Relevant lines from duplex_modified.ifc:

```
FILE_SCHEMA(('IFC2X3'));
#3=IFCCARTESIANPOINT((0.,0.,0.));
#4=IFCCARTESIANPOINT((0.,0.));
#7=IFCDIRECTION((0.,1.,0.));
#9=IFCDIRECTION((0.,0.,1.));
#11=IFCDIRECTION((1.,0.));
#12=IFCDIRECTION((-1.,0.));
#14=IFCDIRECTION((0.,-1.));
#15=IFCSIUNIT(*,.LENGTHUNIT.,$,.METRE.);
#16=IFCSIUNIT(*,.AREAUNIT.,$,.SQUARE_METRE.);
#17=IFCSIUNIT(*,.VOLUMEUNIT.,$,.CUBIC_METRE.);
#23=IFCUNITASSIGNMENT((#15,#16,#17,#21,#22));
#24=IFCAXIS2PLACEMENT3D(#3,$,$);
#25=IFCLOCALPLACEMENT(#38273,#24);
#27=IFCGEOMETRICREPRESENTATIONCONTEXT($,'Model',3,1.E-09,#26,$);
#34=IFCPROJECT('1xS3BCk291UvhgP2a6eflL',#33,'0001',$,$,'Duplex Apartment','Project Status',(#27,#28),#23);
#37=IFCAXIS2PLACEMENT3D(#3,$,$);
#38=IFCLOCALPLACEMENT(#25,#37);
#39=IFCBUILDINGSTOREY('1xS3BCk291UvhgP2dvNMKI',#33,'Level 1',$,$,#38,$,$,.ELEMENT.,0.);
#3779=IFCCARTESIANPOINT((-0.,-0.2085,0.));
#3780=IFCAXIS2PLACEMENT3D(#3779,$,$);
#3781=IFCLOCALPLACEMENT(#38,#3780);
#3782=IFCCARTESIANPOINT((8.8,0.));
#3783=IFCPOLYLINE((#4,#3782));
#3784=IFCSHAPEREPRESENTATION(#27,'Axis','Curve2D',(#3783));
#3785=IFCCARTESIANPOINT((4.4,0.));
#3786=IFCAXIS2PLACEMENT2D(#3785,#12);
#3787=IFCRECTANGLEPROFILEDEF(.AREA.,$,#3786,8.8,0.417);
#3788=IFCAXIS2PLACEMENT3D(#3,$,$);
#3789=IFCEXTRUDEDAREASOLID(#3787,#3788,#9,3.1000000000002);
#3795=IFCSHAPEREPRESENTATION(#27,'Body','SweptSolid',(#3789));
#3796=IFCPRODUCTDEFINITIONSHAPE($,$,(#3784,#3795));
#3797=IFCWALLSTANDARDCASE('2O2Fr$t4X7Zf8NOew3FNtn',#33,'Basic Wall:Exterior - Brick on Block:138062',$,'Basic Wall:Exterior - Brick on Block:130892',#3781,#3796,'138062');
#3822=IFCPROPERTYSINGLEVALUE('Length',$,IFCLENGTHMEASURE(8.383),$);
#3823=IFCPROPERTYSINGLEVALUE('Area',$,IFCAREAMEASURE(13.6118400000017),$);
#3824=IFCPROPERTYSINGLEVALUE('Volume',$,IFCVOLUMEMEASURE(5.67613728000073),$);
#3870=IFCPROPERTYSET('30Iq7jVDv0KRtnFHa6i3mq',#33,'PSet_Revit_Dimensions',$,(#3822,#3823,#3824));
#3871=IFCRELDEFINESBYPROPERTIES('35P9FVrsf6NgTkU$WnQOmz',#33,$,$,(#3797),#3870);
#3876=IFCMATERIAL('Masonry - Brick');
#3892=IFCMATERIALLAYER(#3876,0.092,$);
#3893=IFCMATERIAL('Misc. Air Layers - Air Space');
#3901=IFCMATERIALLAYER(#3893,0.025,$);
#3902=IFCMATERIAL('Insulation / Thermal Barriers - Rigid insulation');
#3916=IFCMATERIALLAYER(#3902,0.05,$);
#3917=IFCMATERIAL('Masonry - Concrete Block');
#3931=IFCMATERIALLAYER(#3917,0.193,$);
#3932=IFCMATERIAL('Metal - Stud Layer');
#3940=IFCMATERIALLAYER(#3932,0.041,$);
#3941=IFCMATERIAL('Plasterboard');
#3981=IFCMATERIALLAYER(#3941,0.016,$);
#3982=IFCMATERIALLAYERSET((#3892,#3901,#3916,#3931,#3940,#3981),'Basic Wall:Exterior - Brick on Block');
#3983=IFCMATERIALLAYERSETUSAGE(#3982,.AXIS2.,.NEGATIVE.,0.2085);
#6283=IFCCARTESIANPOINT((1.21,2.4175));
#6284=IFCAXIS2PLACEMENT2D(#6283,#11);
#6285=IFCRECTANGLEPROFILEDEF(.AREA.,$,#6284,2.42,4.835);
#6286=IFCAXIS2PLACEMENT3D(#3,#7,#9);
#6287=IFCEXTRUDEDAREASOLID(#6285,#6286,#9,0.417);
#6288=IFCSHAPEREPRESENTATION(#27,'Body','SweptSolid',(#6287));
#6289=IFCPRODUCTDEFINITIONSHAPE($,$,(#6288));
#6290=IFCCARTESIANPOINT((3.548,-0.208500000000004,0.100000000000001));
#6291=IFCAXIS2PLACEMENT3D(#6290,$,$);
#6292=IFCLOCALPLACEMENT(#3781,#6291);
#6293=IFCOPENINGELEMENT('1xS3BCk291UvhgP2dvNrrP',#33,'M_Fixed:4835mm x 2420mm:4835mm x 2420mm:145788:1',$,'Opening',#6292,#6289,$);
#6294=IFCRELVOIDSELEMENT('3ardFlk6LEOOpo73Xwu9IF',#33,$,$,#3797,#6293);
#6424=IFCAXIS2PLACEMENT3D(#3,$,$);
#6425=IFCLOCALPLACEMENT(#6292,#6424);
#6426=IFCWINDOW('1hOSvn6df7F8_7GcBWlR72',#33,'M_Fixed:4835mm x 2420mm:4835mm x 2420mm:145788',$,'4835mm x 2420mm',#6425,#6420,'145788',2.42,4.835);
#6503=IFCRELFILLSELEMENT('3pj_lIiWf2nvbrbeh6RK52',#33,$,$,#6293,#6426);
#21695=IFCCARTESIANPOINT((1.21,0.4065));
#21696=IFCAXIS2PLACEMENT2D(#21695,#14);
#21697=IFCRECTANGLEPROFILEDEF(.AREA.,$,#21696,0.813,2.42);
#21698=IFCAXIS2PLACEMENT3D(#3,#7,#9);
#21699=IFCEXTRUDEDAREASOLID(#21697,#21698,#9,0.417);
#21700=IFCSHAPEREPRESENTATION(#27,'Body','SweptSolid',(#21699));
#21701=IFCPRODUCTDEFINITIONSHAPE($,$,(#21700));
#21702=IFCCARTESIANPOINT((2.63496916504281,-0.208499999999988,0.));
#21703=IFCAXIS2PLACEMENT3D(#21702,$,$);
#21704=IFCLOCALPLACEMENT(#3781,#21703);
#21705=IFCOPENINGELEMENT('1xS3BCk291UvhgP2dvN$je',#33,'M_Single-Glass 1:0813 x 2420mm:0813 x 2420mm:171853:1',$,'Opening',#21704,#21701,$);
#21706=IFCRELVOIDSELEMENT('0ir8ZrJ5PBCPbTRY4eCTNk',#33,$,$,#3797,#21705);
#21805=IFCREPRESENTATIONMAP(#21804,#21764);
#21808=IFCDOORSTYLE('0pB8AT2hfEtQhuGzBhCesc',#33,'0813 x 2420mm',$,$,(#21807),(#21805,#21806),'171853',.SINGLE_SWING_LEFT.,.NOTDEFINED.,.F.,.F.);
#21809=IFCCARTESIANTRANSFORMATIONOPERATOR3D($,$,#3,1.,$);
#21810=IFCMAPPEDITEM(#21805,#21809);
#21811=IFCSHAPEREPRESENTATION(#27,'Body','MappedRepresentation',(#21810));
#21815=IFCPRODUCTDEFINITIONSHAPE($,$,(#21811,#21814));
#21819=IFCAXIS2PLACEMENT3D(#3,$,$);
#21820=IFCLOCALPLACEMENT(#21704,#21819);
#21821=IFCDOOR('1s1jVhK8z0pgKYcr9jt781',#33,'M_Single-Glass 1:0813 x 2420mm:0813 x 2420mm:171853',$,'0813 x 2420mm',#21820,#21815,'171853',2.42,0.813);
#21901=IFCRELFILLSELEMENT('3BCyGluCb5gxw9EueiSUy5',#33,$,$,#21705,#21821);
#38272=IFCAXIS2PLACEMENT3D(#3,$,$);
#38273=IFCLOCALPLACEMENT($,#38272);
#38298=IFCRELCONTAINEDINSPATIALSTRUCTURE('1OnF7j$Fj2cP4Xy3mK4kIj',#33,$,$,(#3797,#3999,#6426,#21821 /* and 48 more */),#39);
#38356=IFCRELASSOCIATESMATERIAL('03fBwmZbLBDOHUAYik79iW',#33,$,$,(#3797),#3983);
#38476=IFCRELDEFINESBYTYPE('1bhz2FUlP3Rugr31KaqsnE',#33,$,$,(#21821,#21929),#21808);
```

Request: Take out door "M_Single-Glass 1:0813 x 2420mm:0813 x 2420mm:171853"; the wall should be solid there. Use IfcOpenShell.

```python
import ifcopenshell
import ifcopenshell.api.feature
import ifcopenshell.api.pset
import ifcopenshell.api.root
import ifcopenshell.geom
import ifcopenshell.util.element
import ifcopenshell.util.shape
import ifcopenshell.util.unit

model = ifcopenshell.open("duplex_modified.ifc")
area_scale = ifcopenshell.util.unit.calculate_unit_scale(model, "AREAUNIT")
volume_scale = ifcopenshell.util.unit.calculate_unit_scale(model, "VOLUMEUNIT")
settings = ifcopenshell.geom.settings()


def volume(element):
    """Net volume in cubic metres, openings subtracted."""
    shape = ifcopenshell.geom.create_shape(settings, element)
    return ifcopenshell.util.shape.get_volume(shape.geometry)


door = model.by_guid("1s1jVhK8z0pgKYcr9jt781")
opening = door.FillsVoids[0].RelatingOpeningElement
wall = opening.VoidsElements[0].RelatingBuildingElement
before = volume(wall)

ifcopenshell.api.root.remove_product(model, product=door)
ifcopenshell.api.feature.remove_feature(model, feature=opening)

after = volume(wall)
thickness = 0.417  # wall thickness in metres

# Update the wall's stored quantities.
pset = model.by_id(ifcopenshell.util.element.get_pset(wall, "PSet_Revit_Dimensions", should_inherit=False)["id"])
ifcopenshell.api.pset.edit_pset(model, pset=pset, properties={
    "Area": model.create_entity("IfcAreaMeasure", after / thickness / area_scale),
    "Volume": model.create_entity("IfcVolumeMeasure", after / volume_scale),
})

print(f"wall volume {before:.3f} -> {after:.3f} m3")

model.write("duplex_modified_edited.ifc")
```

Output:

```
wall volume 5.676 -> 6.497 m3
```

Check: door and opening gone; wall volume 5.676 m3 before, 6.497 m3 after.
